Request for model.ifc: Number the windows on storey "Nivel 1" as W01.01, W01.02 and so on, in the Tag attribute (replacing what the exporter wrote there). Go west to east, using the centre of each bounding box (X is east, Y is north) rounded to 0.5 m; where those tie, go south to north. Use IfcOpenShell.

First a look at what the model holds.

```python
import ifcopenshell
import ifcopenshell.util.element
import ifcopenshell.util.placement

model = ifcopenshell.open("model.ifc")
print(model.schema)
storey = next(s for s in model.by_type("IfcBuildingStorey") if s.Name == "Nivel 1")
windows = [e for e in ifcopenshell.util.element.get_decomposition(storey) if e.is_a("IfcWindow")]
for e in sorted(windows, key=lambda e: e.id()):
    origin = ifcopenshell.util.placement.get_local_placement(e.ObjectPlacement)[:3, 3]
    print(e.id(), e.Tag, e.Name, origin.round(2) + 0.0, sep=" | ")
```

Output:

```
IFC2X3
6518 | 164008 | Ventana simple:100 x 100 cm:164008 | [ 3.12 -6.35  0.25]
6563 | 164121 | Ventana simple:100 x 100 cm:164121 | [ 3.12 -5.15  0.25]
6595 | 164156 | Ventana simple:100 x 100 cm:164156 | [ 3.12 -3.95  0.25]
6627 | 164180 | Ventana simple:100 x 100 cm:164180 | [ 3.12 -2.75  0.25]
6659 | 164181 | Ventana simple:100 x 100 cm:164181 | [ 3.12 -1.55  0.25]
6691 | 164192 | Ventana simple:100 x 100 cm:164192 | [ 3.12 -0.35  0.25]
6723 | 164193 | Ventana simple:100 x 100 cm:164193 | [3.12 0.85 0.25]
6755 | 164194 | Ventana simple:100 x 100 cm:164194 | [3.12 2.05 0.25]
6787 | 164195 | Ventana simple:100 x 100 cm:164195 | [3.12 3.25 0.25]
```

```python
import ifcopenshell
import ifcopenshell.geom
import ifcopenshell.util.element
import ifcopenshell.util.shape

model = ifcopenshell.open("model.ifc")
settings = ifcopenshell.geom.settings()
settings.set("use-world-coords", True)


def centre(element):
    shape = ifcopenshell.geom.create_shape(settings, element)
    return ifcopenshell.util.shape.get_bbox_centroid(shape.geometry)


storey = next(s for s in model.by_type("IfcBuildingStorey") if s.Name == "Nivel 1")
windows = [e for e in ifcopenshell.util.element.get_decomposition(storey) if e.is_a("IfcWindow")]

# Insertion points can sit at a corner or the storey origin, so sort by the geometry (in metres).
centres = {e: centre(e) for e in windows}
windows.sort(key=lambda e: (round(centres[e][0] / 0.5), centres[e][1]))

for i, e in enumerate(windows, start=1):
    number = f"W01.{i:02d}"
    e.Tag = number
    print(e.id(), number)

model.write("model_edited.ifc")
```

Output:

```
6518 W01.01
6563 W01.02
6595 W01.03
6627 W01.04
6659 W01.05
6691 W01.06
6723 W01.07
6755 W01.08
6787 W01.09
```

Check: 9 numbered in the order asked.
